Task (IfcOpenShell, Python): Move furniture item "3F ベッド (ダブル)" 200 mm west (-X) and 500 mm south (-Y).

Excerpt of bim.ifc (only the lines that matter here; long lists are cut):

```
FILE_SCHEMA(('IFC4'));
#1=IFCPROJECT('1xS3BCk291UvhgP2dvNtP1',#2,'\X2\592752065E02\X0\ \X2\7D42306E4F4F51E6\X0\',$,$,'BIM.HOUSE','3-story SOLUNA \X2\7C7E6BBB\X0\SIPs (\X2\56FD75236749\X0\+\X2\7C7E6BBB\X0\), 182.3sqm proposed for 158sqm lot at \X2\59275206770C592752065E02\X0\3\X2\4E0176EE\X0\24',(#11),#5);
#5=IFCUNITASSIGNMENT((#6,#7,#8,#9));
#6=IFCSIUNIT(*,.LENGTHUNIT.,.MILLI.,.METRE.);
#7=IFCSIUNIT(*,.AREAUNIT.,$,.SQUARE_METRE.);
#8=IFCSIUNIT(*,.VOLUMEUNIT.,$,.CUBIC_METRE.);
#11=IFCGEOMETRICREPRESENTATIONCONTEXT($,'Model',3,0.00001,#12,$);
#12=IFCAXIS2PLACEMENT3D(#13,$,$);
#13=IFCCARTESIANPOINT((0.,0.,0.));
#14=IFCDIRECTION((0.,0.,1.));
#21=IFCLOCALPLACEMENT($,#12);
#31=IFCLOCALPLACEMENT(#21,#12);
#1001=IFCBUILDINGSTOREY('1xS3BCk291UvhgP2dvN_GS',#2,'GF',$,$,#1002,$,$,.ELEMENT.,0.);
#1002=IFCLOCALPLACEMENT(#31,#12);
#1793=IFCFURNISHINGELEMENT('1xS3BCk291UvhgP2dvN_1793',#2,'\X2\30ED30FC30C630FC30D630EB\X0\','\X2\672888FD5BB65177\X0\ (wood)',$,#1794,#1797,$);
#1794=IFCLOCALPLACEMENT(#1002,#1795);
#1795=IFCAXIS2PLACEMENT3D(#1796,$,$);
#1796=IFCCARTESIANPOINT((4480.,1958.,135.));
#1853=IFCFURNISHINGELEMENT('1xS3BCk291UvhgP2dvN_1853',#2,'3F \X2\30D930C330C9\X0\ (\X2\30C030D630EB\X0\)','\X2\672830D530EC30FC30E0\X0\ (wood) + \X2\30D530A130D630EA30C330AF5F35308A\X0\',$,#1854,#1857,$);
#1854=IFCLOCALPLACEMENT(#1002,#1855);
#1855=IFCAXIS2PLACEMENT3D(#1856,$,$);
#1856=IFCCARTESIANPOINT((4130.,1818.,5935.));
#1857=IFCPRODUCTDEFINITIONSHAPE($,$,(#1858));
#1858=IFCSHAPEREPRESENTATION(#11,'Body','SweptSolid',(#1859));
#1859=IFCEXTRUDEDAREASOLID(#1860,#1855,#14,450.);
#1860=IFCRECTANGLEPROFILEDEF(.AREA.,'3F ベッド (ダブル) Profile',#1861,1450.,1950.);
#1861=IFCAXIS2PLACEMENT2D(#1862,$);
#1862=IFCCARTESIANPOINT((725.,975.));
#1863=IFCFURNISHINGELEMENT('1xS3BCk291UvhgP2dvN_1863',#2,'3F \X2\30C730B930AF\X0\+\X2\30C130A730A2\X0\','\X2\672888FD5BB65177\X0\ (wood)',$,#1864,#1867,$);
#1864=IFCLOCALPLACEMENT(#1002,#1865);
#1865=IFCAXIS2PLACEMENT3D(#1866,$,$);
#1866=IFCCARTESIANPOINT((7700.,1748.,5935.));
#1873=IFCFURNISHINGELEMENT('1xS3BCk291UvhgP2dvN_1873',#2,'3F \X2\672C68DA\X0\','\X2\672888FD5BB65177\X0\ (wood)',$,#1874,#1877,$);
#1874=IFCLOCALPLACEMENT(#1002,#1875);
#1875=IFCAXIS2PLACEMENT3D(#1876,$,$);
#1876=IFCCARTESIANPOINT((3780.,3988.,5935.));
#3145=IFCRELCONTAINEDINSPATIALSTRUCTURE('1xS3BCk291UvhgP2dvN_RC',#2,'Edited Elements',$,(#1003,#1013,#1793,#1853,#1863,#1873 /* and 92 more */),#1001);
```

```python
import ifcopenshell
import ifcopenshell.api.geometry
import ifcopenshell.util.placement
import ifcopenshell.util.unit

model = ifcopenshell.open("bim.ifc")
unit_scale = ifcopenshell.util.unit.calculate_unit_scale(model)

item = model.by_guid("1xS3BCk291UvhgP2dvN_1853")
matrix = ifcopenshell.util.placement.get_local_placement(item.ObjectPlacement)
matrix[0, 3] -= 0.2 / unit_scale
matrix[1, 3] -= 0.5 / unit_scale
ifcopenshell.api.geometry.edit_object_placement(model, product=item, matrix=matrix, is_si=False)

print(ifcopenshell.util.placement.get_local_placement(item.ObjectPlacement).round(3) + 0.0)

model.write("bim_rev.ifc")
```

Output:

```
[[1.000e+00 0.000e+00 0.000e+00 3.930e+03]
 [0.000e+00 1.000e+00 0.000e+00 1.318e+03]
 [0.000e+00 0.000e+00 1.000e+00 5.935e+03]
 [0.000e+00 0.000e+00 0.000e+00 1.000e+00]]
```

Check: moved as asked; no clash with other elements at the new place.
